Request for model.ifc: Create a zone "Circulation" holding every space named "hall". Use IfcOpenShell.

First a look at what the model holds.

```python
import ifcopenshell

model = ifcopenshell.open("model.ifc")
print(model.schema)
seen = {}
for space in model.by_type("IfcSpace"):
    seen[space.LongName] = seen.get(space.LongName, 0) + 1
for name, count in sorted(seen.items(), key=str):
    print(count, "x", name)
print("zones:", [z.Name for z in model.by_type("IfcZone")][:20])
```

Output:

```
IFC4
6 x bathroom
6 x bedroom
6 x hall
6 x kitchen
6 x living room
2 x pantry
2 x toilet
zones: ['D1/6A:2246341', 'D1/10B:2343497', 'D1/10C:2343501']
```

```python
import ifcopenshell
import ifcopenshell.api.group
import ifcopenshell.api.root

model = ifcopenshell.open("model.ifc")

names = {"hall"}
spaces = [s for s in model.by_type("IfcSpace") if s.LongName in names]

zone = ifcopenshell.api.root.create_entity(model, ifc_class="IfcZone", name="Circulation")
ifcopenshell.api.group.assign_group(model, products=spaces, group=zone)
print(len(spaces), "spaces in", zone.Name)

model.write("model_rev.ifc")
```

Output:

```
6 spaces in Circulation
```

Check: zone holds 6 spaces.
